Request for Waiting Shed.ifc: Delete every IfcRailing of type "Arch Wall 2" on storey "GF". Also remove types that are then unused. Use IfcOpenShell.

First a look at what the model holds.

```python
import ifcopenshell
import ifcopenshell.util.element

model = ifcopenshell.open("Waiting Shed.ifc")
print(model.schema)
storey = next(s for s in model.by_type("IfcBuildingStorey") if s.Name == "GF")
railings = [e for e in ifcopenshell.util.element.get_decomposition(storey) if e.is_a("IfcRailing")]
seen = {}
for e in railings:
    element_type = ifcopenshell.util.element.get_type(e)
    name = element_type.Name if element_type not in (None, e) else None
    seen[name] = seen.get(name, 0) + 1
for name, count in sorted(seen.items(), key=str):
    print(count, "x", name)
```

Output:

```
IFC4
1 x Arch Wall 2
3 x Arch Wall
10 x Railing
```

```python
import ifcopenshell
import ifcopenshell.api.root
import ifcopenshell.util.element

model = ifcopenshell.open("Waiting Shed.ifc")

storey = next(s for s in model.by_type("IfcBuildingStorey") if s.Name == "GF")
railings = [e for e in ifcopenshell.util.element.get_decomposition(storey) if e.is_a("IfcRailing")]
targets = [e for e in railings if (t := ifcopenshell.util.element.get_type(e)) not in (None, e) and t.Name == "Arch Wall 2"]
types = {ifcopenshell.util.element.get_type(e) for e in targets} - {None, *targets}

for e in targets:
    ifcopenshell.api.root.remove_product(model, product=e)
print(len(targets), "removed")

unused = [t for t in types if not ifcopenshell.util.element.get_types(t)]
for t in unused:
    ifcopenshell.api.root.remove_product(model, product=t)
print(len(unused), "unused types removed")

model.write("Waiting Shed_edited.ifc")
```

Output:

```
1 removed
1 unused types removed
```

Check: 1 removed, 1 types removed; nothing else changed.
